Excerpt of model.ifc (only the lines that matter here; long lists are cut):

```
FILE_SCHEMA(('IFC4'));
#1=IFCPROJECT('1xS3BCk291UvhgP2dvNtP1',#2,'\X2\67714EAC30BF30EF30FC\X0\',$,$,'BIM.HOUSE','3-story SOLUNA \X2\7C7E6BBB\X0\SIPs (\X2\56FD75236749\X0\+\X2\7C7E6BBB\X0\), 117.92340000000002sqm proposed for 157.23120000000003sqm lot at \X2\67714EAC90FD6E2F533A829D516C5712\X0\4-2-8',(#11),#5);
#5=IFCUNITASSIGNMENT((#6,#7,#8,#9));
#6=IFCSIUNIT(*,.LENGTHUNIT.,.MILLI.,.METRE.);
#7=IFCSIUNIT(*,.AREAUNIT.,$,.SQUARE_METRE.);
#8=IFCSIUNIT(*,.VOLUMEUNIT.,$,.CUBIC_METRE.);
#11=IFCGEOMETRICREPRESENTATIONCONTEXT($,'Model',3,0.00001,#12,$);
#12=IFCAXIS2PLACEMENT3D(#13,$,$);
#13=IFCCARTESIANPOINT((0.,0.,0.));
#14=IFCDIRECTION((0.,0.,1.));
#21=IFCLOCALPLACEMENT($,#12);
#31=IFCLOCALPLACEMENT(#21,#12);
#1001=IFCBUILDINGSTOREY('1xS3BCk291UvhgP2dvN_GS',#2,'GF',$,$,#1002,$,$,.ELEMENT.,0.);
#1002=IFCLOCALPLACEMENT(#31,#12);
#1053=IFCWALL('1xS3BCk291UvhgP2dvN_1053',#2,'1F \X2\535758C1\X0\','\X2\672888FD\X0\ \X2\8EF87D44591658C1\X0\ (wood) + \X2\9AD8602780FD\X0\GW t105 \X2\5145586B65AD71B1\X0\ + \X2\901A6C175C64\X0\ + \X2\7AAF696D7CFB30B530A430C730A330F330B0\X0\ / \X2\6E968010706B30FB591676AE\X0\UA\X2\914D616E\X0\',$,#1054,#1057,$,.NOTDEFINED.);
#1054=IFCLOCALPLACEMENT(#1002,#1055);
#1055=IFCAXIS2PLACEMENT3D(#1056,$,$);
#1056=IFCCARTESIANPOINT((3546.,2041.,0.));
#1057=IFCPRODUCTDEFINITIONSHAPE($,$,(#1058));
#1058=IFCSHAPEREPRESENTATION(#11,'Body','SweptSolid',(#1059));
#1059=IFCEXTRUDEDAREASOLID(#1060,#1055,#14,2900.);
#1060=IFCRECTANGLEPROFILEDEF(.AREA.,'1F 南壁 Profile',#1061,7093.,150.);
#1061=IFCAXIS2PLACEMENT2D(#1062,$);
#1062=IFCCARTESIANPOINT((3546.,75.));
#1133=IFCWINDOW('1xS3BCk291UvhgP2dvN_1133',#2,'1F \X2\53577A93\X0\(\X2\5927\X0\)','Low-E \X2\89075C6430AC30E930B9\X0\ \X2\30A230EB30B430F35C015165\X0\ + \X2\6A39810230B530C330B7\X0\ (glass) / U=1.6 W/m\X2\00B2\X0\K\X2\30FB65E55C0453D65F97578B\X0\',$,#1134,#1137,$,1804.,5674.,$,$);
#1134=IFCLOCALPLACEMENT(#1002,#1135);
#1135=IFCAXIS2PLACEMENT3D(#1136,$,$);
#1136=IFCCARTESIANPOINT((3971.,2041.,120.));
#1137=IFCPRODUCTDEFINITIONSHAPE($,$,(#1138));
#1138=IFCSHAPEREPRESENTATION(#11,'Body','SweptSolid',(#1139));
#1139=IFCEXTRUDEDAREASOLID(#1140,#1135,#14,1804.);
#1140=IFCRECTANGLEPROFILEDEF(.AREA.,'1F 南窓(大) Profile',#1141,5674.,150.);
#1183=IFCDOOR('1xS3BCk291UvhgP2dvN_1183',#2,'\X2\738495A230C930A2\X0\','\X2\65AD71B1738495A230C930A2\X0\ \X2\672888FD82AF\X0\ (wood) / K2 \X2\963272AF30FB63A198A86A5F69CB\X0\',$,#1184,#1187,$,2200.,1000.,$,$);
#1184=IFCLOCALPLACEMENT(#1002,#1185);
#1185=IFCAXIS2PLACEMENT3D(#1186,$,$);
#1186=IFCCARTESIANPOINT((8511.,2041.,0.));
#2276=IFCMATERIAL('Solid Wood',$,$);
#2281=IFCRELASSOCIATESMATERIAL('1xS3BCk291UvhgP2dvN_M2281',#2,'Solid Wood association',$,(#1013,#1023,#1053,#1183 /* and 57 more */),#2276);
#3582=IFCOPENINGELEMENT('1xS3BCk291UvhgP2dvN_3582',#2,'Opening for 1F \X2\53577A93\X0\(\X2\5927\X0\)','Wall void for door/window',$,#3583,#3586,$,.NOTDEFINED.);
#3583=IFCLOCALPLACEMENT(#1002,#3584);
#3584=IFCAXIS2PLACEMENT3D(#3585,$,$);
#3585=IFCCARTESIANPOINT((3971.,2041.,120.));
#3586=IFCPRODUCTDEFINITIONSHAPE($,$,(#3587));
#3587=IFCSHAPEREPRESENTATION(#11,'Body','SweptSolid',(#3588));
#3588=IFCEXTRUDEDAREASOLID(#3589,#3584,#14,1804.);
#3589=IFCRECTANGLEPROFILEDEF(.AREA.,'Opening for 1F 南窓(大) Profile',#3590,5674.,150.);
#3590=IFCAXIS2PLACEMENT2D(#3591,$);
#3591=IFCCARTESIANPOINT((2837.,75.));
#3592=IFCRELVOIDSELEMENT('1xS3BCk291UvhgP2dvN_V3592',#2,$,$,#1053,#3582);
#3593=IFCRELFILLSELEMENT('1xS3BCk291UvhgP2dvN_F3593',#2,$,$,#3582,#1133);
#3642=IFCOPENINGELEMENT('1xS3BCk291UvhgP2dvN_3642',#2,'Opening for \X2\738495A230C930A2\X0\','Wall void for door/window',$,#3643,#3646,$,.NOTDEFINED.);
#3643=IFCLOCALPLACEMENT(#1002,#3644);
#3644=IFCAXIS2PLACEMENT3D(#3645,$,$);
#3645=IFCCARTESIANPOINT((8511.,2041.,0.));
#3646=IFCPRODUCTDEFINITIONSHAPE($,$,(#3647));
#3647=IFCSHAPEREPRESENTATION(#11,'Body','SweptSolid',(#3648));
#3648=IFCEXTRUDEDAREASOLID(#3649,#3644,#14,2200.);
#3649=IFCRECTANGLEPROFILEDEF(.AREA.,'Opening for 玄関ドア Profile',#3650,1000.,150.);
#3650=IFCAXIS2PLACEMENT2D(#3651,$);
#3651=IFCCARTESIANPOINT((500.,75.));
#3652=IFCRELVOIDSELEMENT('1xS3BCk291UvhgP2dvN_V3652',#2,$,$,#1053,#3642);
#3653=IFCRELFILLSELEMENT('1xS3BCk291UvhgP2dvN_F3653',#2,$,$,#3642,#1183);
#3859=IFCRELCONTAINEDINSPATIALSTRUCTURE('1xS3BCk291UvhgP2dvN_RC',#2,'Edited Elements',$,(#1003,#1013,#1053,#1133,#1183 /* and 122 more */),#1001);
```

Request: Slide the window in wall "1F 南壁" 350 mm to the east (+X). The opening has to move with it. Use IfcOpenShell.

```python
import ifcopenshell
import ifcopenshell.api.geometry
import ifcopenshell.util.placement
import ifcopenshell.util.unit

model = ifcopenshell.open("model.ifc")
unit_scale = ifcopenshell.util.unit.calculate_unit_scale(model)

window = model.by_id(1133)
opening = window.FillsVoids[0].RelatingOpeningElement
wall = opening.VoidsElements[0].RelatingBuildingElement

wall_matrix = ifcopenshell.util.placement.get_local_placement(wall.ObjectPlacement)
shift = wall_matrix[:3, 0] * 0.35 / unit_scale
before = ifcopenshell.util.placement.get_local_placement(window.ObjectPlacement)[:3, 3].copy()

# The window is not placed relative to its opening, so move both.
for product in (opening, window):
    matrix = ifcopenshell.util.placement.get_local_placement(product.ObjectPlacement)
    matrix[:3, 3] += shift
    ifcopenshell.api.geometry.edit_object_placement(model, product=product, matrix=matrix, is_si=False)

after = ifcopenshell.util.placement.get_local_placement(window.ObjectPlacement)[:3, 3]
print("window moved by", (after - before).round(3) + 0.0)

model.write("model_rev.ifc")
```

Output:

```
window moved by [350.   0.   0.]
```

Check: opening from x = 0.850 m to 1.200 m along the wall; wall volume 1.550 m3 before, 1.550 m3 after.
